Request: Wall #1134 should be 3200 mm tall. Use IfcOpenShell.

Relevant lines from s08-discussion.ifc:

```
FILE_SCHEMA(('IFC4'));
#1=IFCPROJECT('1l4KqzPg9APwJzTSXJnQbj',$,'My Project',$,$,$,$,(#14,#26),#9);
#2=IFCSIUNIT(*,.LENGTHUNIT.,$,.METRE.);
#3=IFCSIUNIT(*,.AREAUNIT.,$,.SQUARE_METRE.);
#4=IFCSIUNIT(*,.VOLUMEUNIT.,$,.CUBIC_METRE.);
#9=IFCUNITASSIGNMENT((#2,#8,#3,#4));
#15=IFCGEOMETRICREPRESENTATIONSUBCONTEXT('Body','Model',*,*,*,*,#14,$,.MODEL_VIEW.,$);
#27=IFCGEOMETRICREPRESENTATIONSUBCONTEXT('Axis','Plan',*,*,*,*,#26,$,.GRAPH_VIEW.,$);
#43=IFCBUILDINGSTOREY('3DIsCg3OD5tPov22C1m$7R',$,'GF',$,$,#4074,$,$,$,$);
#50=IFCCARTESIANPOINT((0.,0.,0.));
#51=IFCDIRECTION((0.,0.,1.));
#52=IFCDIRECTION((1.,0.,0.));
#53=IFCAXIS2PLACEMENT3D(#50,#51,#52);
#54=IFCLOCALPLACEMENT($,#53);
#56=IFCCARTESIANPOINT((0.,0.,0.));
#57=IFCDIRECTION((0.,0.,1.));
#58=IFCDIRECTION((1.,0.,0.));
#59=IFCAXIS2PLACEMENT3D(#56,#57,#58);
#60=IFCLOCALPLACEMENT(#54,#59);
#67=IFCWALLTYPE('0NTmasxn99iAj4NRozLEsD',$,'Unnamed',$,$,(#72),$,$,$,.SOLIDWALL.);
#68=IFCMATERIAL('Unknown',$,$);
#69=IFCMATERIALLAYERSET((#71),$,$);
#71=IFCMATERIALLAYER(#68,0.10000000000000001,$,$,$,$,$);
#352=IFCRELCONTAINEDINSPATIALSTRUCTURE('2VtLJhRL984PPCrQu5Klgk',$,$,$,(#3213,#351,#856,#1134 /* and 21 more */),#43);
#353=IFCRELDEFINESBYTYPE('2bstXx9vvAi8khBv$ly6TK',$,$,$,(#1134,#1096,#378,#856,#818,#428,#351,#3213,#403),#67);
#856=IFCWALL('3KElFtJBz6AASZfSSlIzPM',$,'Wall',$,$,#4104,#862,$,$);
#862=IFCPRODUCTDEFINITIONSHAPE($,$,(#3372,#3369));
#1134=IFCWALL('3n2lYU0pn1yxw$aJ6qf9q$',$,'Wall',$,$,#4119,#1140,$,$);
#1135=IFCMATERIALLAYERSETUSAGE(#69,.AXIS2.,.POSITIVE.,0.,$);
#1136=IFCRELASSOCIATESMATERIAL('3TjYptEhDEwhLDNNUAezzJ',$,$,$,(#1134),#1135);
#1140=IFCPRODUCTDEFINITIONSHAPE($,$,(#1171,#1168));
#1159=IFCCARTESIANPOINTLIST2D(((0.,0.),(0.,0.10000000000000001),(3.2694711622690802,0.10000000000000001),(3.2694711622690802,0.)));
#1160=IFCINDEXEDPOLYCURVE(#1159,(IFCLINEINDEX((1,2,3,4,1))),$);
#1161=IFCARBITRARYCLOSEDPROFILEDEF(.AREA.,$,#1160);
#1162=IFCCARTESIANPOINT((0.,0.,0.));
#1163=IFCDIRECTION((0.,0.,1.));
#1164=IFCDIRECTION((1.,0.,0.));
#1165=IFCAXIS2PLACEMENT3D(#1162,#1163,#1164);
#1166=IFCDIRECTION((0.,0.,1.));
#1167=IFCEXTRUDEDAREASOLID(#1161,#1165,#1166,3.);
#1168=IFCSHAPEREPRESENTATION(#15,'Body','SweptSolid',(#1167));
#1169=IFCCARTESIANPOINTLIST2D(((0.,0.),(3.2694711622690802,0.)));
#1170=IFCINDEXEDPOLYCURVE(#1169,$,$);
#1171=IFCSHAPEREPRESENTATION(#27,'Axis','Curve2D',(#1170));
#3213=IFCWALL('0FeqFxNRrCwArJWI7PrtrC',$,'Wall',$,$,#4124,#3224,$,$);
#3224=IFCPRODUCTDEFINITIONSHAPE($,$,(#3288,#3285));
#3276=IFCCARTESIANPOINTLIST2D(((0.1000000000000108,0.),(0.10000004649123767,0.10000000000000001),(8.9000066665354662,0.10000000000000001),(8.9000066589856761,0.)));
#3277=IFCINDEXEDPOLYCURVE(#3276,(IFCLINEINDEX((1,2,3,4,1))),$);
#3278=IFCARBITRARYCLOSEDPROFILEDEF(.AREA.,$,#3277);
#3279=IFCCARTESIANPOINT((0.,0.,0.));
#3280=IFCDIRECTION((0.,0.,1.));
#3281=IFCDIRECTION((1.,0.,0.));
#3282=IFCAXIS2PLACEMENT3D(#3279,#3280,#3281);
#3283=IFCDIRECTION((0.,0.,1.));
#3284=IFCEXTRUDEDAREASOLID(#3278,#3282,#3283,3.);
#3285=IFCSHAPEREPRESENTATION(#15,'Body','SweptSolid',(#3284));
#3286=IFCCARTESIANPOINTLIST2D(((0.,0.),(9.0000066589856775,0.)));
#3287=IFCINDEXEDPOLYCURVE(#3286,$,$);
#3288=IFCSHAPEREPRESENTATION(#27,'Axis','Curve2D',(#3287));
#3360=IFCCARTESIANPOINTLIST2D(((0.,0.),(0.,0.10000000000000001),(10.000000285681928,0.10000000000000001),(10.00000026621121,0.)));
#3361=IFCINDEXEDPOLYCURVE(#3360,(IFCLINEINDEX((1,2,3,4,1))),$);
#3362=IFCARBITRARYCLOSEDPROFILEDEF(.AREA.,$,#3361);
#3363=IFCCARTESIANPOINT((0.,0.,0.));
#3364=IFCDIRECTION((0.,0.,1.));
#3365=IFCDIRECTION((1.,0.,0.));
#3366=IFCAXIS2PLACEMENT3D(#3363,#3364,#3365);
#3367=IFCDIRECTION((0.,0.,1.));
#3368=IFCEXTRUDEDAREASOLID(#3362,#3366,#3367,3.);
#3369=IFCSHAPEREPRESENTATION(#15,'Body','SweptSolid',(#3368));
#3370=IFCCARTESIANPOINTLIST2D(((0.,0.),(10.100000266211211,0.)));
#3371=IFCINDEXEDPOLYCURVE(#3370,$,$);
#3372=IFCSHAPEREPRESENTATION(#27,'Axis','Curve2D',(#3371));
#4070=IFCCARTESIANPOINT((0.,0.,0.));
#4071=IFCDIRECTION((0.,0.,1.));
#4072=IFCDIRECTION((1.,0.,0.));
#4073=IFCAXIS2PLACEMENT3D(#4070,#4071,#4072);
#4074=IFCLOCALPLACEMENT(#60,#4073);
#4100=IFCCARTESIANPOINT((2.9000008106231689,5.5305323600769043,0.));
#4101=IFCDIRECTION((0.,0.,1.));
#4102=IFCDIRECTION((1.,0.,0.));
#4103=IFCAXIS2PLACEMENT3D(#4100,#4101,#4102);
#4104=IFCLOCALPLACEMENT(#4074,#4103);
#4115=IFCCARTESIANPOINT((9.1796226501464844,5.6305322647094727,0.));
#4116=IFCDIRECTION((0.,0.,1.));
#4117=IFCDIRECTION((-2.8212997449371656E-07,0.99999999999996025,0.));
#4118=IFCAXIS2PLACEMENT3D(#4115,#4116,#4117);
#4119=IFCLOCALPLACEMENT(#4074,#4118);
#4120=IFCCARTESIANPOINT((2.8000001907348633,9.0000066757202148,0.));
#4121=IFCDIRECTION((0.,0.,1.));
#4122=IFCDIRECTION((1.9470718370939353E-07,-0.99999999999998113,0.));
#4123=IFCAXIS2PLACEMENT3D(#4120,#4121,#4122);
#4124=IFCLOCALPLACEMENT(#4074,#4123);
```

```python
import ifcopenshell
import ifcopenshell.geom
import ifcopenshell.util.representation
import ifcopenshell.util.shape
import ifcopenshell.util.unit

model = ifcopenshell.open("s08-discussion.ifc")
unit_scale = ifcopenshell.util.unit.calculate_unit_scale(model)
settings = ifcopenshell.geom.settings()


def volume(element):
    """Net volume in cubic metres, openings subtracted."""
    shape = ifcopenshell.geom.create_shape(settings, element)
    return ifcopenshell.util.shape.get_volume(shape.geometry)


wall = model.by_guid("3n2lYU0pn1yxw$aJ6qf9q$")
before = volume(wall)

body = ifcopenshell.util.representation.get_representation(wall, "Model", "Body")
solid = body.Items[0]
old_height = solid.Depth
solid.Depth = 3.2 / unit_scale
after = volume(wall)

print(f"height {old_height:g} -> {solid.Depth:g}, volume {before:.3f} -> {after:.3f} m3")

model.write("s08-discussion_v2.ifc")
```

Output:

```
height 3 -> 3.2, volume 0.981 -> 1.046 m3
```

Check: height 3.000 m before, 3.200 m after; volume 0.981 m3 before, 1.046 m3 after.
